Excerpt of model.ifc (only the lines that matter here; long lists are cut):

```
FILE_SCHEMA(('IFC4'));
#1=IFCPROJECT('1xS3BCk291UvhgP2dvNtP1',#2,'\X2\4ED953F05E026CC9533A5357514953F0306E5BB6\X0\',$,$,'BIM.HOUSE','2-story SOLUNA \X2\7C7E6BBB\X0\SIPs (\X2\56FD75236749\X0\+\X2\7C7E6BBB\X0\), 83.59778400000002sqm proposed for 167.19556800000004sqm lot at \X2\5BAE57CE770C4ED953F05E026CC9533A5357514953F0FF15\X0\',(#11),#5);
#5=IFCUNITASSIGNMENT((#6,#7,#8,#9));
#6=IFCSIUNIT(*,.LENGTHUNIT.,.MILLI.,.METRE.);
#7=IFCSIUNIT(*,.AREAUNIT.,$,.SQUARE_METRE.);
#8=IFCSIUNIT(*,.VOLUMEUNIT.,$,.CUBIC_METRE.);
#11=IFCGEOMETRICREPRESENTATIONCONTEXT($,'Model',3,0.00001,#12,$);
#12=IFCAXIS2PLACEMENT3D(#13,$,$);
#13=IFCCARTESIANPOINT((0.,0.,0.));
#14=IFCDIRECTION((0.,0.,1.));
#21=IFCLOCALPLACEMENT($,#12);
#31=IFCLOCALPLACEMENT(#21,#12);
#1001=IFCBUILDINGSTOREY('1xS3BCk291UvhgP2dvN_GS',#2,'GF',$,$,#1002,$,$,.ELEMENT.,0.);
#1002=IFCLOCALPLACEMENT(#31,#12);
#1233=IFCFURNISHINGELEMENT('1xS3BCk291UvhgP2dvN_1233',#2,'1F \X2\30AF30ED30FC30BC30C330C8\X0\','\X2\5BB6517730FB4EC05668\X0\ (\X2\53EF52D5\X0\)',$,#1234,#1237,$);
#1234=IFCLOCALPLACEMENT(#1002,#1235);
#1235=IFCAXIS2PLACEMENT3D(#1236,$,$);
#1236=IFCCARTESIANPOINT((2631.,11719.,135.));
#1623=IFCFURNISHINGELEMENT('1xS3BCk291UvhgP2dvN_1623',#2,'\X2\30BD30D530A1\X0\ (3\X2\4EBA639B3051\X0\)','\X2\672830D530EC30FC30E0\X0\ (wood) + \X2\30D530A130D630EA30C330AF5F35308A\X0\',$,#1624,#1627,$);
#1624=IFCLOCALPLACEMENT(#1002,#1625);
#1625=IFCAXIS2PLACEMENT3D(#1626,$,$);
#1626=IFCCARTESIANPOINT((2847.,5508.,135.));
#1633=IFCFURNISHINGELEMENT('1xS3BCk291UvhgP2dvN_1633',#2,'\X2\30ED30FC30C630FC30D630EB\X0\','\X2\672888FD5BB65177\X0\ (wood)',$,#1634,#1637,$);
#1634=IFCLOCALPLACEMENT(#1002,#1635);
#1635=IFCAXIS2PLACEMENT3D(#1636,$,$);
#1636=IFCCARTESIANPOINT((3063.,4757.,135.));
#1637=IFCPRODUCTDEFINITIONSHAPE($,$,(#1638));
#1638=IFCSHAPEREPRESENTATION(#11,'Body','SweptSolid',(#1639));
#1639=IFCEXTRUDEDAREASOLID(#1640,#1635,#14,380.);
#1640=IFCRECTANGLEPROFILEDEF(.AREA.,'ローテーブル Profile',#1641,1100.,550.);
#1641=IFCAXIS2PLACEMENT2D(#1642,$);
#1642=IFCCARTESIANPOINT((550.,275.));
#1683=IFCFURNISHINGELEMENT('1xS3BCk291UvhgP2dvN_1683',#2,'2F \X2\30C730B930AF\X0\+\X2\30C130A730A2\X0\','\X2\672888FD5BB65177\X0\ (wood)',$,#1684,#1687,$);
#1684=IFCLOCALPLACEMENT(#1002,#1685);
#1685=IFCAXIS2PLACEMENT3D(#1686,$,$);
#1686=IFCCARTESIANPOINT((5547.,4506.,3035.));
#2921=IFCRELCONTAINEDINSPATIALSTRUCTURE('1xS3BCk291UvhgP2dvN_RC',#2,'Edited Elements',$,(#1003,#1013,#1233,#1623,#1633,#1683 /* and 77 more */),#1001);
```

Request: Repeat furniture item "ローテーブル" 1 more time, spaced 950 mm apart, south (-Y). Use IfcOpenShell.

```python
import numpy as np
import ifcopenshell
import ifcopenshell.api.geometry
import ifcopenshell.api.root
import ifcopenshell.util.element
import ifcopenshell.util.placement
import ifcopenshell.util.unit

model = ifcopenshell.open("model.ifc")
unit_scale = ifcopenshell.util.unit.calculate_unit_scale(model)


def reuse_history(source, copy):
    """copy_class also copies each property set's owner history, people and application; keep the originals."""
    for rel in copy.IsDefinedBy:
        if rel.is_a("IfcRelDefinesByProperties") and (history := rel.RelatingPropertyDefinition.OwnerHistory):
            rel.RelatingPropertyDefinition.OwnerHistory = source.OwnerHistory
            ifcopenshell.util.element.remove_deep2(model, history)


source = model.by_guid("1xS3BCk291UvhgP2dvN_1633")
base = ifcopenshell.util.placement.get_local_placement(source.ObjectPlacement)
step = np.array([0.0, -1.0, 0.0]) * 0.95 / unit_scale

for i in range(1, 2):
    copy = ifcopenshell.api.root.copy_class(model, product=source)
    copy.Representation = ifcopenshell.util.element.copy_deep(
        model, source.Representation, exclude=["IfcGeometricRepresentationContext", "IfcRepresentationMap"]
    )
    reuse_history(source, copy)
    matrix = base.copy()
    matrix[:3, 3] += i * step
    print("added at", matrix[:3, 3].round(3) + 0.0)
    ifcopenshell.api.geometry.edit_object_placement(model, product=copy, matrix=matrix, is_si=False)

model.write("model-out.ifc")
```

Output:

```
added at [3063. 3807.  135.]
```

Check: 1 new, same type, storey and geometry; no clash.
